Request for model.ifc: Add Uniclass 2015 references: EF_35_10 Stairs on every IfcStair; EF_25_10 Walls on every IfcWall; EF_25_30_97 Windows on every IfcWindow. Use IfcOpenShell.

First a look at what the model holds.

```python
import ifcopenshell

model = ifcopenshell.open("model.ifc")
print(model.schema)
print("classifications:", [c.Name for c in model.by_type("IfcClassification")])
for ifc_class in ("IfcDoor", "IfcRoof", "IfcStair", "IfcWall", "IfcWindow"):
    print(ifc_class, len(model.by_type(ifc_class)))
```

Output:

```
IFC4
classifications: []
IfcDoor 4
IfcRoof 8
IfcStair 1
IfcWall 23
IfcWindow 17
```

```python
import ifcopenshell
import ifcopenshell.api.classification

model = ifcopenshell.open("model.ifc")

system = ifcopenshell.api.classification.add_classification(model, classification="Uniclass 2015")

codes = {
    "IfcStair": ("EF_35_10", "Stairs"),
    "IfcWall": ("EF_25_10", "Walls"),
    "IfcWindow": ("EF_25_30_97", "Windows"),
}
for ifc_class, (code, name) in codes.items():
    products = model.by_type(ifc_class)
    ifcopenshell.api.classification.add_reference(
        model, products=products, classification=system, identification=code, name=name
    )
    print(code, len(products))

model.write("model_updated.ifc")
```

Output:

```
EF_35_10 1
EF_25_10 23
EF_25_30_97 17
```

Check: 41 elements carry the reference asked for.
